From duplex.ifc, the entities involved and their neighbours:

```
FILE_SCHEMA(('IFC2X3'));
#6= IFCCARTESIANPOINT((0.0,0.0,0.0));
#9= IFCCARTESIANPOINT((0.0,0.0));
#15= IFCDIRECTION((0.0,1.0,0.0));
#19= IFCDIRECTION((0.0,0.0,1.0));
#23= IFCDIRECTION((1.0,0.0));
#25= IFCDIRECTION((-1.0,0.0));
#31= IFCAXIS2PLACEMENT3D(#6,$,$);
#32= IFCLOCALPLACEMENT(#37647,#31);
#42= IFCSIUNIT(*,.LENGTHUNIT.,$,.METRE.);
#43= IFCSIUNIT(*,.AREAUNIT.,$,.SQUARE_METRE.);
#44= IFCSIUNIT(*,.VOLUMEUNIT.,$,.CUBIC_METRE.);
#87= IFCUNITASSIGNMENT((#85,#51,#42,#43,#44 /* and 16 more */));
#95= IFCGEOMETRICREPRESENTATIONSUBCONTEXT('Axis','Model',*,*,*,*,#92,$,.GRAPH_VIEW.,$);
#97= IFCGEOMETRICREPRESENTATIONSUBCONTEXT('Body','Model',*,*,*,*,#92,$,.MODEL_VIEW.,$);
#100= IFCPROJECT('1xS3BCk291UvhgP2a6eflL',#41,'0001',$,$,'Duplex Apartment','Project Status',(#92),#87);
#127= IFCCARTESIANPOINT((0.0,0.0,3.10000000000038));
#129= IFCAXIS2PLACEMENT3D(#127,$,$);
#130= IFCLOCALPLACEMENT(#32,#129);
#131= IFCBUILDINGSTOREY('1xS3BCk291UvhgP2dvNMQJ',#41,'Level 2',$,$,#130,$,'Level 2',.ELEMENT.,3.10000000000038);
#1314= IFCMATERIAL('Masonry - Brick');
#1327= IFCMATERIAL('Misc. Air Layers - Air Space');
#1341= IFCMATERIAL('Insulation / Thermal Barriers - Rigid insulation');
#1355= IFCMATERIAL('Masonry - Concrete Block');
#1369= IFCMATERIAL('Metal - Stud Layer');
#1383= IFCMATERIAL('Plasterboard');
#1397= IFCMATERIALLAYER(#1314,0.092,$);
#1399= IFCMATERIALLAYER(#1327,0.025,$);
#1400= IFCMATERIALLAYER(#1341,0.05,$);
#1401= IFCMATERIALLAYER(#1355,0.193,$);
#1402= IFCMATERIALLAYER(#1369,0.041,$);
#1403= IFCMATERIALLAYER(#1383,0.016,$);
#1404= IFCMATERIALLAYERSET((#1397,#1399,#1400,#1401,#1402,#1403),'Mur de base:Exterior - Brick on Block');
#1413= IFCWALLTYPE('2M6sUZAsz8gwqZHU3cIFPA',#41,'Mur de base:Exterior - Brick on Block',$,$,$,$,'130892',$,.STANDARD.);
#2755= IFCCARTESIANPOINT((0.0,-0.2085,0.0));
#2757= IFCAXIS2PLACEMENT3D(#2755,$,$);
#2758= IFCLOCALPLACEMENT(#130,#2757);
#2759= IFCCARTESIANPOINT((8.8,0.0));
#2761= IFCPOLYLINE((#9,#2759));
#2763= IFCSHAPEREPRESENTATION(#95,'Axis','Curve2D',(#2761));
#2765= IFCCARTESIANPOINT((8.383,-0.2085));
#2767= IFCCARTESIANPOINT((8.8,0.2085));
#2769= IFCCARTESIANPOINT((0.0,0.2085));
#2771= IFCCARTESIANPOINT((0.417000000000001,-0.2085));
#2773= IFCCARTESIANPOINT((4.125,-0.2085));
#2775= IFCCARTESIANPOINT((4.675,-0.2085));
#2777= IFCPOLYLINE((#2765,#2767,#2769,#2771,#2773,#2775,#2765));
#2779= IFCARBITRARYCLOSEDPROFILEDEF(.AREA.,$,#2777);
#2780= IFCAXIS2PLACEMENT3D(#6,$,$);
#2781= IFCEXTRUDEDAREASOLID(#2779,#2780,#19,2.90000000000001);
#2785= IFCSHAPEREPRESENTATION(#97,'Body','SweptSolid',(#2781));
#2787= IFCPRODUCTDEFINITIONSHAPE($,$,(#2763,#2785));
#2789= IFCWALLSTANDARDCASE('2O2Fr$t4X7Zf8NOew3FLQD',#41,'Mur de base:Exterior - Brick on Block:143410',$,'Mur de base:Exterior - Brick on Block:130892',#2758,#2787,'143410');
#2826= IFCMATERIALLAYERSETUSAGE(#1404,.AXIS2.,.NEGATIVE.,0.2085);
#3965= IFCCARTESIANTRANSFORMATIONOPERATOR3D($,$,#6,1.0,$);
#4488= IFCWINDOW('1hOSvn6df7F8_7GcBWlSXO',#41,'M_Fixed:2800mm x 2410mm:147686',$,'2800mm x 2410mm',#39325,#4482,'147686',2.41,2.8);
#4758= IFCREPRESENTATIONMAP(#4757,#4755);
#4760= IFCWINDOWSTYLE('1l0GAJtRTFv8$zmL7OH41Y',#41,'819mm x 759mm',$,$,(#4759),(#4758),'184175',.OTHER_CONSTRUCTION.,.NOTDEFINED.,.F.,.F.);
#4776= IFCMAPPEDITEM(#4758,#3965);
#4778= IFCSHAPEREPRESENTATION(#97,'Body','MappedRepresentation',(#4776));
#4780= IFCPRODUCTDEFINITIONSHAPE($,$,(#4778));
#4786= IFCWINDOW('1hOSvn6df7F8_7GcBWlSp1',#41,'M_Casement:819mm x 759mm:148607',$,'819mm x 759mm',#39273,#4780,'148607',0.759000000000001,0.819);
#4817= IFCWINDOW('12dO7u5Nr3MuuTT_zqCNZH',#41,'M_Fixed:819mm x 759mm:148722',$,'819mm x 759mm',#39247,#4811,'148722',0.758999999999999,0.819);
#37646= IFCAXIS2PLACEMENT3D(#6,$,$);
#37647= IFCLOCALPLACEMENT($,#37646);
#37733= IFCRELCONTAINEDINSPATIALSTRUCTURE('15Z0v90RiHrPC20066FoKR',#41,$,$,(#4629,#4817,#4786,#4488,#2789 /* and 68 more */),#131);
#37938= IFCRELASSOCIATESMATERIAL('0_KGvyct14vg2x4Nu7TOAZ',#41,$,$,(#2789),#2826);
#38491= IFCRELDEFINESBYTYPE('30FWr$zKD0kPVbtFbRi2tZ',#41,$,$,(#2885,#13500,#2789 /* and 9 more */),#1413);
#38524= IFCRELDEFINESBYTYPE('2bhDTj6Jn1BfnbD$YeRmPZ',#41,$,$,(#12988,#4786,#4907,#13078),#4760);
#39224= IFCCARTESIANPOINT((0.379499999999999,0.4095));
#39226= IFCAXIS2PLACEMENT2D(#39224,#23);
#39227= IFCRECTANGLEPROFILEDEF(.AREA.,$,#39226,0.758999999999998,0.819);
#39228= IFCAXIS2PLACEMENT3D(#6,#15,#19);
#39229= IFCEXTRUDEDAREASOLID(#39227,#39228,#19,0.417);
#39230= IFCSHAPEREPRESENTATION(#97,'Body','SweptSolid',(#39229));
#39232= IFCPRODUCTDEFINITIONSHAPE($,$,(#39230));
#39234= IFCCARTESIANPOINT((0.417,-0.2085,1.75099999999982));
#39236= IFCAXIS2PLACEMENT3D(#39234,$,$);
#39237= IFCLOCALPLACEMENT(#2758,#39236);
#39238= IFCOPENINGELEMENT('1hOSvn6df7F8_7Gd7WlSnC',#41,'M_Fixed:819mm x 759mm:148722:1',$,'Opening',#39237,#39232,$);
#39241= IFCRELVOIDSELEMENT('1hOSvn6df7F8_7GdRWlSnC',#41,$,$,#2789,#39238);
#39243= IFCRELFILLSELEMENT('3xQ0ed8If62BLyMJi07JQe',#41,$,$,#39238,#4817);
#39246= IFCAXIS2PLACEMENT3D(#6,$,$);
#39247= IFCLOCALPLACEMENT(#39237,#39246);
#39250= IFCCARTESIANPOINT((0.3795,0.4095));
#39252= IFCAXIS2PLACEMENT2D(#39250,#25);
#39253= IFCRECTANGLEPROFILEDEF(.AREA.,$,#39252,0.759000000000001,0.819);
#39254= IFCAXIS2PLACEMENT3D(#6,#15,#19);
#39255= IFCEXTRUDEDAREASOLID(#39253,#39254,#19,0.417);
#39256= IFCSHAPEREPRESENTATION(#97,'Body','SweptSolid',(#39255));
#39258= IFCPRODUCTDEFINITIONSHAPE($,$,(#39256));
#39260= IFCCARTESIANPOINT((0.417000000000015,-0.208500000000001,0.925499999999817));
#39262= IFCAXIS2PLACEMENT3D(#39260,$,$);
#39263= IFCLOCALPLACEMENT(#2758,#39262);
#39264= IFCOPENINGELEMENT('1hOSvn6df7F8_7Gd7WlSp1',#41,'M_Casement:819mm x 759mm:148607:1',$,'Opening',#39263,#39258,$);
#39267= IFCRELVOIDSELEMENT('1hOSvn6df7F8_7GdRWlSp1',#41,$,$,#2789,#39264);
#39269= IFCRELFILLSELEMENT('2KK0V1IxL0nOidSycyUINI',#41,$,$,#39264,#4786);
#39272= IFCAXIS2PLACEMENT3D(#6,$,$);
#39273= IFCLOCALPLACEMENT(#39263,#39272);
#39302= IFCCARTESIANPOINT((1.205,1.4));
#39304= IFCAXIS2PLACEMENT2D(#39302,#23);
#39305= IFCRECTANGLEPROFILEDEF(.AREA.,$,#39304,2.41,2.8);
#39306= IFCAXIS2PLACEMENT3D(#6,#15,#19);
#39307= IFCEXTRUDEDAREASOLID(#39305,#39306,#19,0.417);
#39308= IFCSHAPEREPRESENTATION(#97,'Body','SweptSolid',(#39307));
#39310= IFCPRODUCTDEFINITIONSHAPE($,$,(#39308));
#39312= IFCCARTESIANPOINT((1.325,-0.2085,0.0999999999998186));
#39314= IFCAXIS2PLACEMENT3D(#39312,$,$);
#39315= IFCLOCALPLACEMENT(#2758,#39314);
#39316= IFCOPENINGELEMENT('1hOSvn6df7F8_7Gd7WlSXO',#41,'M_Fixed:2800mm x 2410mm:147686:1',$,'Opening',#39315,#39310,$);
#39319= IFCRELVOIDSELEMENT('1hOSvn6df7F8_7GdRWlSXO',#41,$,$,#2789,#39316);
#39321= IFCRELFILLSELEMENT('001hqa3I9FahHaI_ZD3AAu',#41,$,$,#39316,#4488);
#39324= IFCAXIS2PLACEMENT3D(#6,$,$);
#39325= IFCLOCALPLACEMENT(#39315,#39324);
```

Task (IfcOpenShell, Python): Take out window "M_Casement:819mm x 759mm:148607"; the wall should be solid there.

```python
import ifcopenshell
import ifcopenshell.api.feature
import ifcopenshell.api.root
import ifcopenshell.geom
import ifcopenshell.util.shape

model = ifcopenshell.open("duplex.ifc")
settings = ifcopenshell.geom.settings()


def volume(element):
    """Net volume in cubic metres, openings subtracted."""
    shape = ifcopenshell.geom.create_shape(settings, element)
    return ifcopenshell.util.shape.get_volume(shape.geometry)


window = model.by_guid("1hOSvn6df7F8_7GcBWlSp1")
opening = window.FillsVoids[0].RelatingOpeningElement
wall = opening.VoidsElements[0].RelatingBuildingElement
before = volume(wall)

ifcopenshell.api.root.remove_product(model, product=window)
ifcopenshell.api.feature.remove_feature(model, feature=opening)

after = volume(wall)

print(f"wall volume {before:.3f} -> {after:.3f} m3")

model.write("duplex-out.ifc")
```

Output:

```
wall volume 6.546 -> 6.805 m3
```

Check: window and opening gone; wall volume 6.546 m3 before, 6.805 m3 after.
